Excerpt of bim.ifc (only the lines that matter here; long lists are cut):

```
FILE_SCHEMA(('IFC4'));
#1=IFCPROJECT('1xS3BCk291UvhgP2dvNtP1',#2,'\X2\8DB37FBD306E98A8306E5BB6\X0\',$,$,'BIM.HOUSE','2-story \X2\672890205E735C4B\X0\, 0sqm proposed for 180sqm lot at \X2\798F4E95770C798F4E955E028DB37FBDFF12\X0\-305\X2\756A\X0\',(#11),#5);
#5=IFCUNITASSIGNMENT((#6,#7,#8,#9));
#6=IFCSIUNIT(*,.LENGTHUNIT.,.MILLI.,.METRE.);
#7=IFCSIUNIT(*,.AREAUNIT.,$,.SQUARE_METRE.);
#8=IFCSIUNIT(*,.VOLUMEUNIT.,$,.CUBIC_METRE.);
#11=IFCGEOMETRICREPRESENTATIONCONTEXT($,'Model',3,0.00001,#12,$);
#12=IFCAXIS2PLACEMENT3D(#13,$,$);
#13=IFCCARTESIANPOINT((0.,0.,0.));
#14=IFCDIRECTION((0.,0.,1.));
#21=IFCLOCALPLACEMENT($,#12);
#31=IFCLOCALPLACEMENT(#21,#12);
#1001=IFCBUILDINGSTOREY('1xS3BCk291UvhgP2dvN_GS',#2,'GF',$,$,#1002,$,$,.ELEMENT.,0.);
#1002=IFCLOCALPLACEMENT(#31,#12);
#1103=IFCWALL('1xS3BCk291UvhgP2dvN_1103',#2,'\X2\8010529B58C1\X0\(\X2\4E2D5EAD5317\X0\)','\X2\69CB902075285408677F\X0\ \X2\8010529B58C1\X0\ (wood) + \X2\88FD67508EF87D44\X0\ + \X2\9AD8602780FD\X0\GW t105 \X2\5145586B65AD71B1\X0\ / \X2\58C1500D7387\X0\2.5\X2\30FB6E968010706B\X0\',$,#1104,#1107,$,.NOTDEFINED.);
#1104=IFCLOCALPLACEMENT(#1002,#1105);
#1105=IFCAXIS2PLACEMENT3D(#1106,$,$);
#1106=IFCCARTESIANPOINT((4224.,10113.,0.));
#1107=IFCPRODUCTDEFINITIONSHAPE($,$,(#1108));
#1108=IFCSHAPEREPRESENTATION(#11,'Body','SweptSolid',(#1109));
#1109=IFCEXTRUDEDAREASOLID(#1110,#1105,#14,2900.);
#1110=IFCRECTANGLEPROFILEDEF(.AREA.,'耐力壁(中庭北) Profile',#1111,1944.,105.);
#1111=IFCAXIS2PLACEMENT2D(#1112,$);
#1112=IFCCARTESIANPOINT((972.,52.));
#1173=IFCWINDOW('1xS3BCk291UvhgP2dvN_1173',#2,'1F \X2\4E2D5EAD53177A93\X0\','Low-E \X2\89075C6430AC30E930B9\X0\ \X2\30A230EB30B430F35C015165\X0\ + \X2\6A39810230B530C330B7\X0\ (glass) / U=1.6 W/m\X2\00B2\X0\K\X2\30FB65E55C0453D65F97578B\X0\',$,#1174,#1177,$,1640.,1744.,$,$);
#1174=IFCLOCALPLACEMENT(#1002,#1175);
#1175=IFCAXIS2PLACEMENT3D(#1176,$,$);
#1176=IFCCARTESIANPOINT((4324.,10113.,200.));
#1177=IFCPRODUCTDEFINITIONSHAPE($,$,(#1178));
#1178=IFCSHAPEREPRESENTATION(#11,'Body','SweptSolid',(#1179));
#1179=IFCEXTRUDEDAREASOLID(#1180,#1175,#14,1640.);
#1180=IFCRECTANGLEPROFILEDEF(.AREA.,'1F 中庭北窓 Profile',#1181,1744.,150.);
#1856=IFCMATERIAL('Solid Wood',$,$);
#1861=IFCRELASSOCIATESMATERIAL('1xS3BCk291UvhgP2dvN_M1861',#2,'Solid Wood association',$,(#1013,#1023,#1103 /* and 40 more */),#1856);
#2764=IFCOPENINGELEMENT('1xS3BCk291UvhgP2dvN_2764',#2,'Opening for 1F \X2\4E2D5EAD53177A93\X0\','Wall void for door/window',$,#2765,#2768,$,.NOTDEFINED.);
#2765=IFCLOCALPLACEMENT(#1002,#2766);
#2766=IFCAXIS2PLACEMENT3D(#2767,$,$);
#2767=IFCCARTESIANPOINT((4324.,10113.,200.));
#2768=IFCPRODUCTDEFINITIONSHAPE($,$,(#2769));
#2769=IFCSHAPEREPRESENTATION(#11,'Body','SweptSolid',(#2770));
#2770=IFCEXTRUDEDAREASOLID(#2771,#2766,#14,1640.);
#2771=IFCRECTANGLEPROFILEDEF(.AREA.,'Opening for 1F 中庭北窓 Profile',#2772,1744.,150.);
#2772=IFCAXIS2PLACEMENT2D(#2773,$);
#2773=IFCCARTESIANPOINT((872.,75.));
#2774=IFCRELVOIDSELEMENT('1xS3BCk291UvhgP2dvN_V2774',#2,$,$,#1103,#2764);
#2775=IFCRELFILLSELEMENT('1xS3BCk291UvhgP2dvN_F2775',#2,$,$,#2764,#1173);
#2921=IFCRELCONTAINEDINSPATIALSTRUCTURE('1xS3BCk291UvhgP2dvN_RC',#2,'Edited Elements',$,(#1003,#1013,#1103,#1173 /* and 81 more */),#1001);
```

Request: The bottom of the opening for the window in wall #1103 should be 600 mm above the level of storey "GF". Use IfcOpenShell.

```python
import numpy as np
import ifcopenshell
import ifcopenshell.api.geometry
import ifcopenshell.geom
import ifcopenshell.util.element
import ifcopenshell.util.placement
import ifcopenshell.util.shape
import ifcopenshell.util.unit

model = ifcopenshell.open("bim.ifc")
unit_scale = ifcopenshell.util.unit.calculate_unit_scale(model)

window = model.by_guid("1xS3BCk291UvhgP2dvN_1173")
opening = window.FillsVoids[0].RelatingOpeningElement
storey = ifcopenshell.util.element.get_container(window, ifc_class="IfcBuildingStorey")
level = ifcopenshell.util.placement.get_local_placement(storey.ObjectPlacement)[2, 3]

# The opening's origin need not be at the sill, so measure its lowest point.
shape = ifcopenshell.geom.create_shape(ifcopenshell.geom.settings(), opening)
bottom = ifcopenshell.util.shape.get_shape_bottom_elevation(shape, shape.geometry) / unit_scale
dz = level + 0.6 / unit_scale - bottom

shift = np.array([0.0, 0.0, dz])
# The window is not placed relative to its opening, so move both.
for product in (opening, window):
    matrix = ifcopenshell.util.placement.get_local_placement(product.ObjectPlacement)
    matrix[:3, 3] += shift
    ifcopenshell.api.geometry.edit_object_placement(model, product=product, matrix=matrix, is_si=False)

print(f"moved by {dz * unit_scale:+.3f} m")

model.write("bim_v2.ifc")
```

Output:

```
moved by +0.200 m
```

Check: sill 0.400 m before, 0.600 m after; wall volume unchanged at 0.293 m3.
